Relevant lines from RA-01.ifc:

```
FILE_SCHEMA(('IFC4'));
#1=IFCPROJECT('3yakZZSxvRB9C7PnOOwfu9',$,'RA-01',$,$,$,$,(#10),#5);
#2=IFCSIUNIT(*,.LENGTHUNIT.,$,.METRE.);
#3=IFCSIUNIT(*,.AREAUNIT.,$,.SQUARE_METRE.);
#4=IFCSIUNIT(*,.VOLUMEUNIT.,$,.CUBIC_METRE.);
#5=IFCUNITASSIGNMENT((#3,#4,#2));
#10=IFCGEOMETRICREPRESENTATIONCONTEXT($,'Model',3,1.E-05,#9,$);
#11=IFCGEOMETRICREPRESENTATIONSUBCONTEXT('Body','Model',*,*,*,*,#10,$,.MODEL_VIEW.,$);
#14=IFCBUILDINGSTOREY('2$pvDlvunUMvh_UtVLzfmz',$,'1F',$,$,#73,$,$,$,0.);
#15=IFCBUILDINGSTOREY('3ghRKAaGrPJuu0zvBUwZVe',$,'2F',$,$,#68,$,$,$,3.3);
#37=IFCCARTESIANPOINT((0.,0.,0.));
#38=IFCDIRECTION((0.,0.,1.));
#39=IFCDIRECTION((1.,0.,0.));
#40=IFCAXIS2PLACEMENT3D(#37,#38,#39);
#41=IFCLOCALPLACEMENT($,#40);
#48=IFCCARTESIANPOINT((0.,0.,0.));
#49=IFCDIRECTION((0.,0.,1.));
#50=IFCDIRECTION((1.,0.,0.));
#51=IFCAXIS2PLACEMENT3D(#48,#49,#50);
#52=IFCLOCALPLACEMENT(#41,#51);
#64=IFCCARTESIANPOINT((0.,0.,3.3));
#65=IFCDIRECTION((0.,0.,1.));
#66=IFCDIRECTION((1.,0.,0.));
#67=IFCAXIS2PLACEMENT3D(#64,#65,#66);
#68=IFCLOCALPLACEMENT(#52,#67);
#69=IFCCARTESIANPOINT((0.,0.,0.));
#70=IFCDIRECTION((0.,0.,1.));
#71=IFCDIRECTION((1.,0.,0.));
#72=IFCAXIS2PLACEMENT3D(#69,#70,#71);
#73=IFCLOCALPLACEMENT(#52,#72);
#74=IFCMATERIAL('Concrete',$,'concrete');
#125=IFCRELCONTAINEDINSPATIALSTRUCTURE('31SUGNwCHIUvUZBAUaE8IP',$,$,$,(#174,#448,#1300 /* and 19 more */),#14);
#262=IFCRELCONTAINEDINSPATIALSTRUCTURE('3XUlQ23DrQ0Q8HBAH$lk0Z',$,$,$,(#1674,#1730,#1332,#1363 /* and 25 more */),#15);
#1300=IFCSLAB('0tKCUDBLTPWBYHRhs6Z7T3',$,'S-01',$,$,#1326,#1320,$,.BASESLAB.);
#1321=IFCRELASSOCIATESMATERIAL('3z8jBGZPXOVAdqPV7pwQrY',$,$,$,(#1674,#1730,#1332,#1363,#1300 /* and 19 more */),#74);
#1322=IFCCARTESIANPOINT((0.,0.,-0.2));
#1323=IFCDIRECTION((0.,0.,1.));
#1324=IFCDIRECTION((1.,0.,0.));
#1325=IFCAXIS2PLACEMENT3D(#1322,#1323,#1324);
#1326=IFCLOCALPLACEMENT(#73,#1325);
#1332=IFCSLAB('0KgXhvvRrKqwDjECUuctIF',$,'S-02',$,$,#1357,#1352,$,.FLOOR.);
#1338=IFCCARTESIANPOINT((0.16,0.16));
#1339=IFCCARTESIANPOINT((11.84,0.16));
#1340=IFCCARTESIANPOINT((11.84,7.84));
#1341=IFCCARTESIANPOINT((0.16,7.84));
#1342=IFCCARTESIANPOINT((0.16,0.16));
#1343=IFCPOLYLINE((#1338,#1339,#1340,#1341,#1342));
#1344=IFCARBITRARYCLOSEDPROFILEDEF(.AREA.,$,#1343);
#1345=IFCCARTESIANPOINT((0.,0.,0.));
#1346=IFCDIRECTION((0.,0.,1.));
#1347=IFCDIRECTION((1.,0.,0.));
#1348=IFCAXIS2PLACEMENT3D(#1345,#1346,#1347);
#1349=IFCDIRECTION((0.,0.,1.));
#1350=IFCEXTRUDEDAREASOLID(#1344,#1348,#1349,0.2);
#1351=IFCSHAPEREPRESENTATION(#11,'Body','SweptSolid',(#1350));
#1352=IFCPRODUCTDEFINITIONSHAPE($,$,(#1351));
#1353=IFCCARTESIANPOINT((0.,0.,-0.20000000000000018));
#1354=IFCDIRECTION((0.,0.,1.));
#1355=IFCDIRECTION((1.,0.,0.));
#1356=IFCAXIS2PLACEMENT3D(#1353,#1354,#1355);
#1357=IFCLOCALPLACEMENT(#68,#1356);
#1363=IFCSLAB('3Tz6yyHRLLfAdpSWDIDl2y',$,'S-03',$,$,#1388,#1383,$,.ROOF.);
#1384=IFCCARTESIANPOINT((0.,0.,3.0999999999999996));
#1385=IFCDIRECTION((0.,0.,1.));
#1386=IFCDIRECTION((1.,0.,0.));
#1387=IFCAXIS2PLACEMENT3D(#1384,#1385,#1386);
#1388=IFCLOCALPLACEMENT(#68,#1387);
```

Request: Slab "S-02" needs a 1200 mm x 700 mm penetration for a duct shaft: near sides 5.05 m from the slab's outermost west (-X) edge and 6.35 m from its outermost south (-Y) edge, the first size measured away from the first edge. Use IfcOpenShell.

```python
import numpy as np
import ifcopenshell
import ifcopenshell.api.feature
import ifcopenshell.api.geometry
import ifcopenshell.api.root
import ifcopenshell.geom
import ifcopenshell.util.placement
import ifcopenshell.util.representation
import ifcopenshell.util.shape
import ifcopenshell.util.unit

model = ifcopenshell.open("RA-01.ifc")
unit_scale = ifcopenshell.util.unit.calculate_unit_scale(model)
settings = ifcopenshell.geom.settings()


def volume(element):
    """Net volume in cubic metres, openings subtracted."""
    shape = ifcopenshell.geom.create_shape(settings, element)
    return ifcopenshell.util.shape.get_volume(shape.geometry)


slab = model.by_guid("0KgXhvvRrKqwDjECUuctIF")
before = volume(slab)

# Extent in the slab's own axes, in metres. The edges named are its -X and -Y sides.
slab_shape = ifcopenshell.geom.create_shape(settings, slab)
vertices = ifcopenshell.util.shape.get_vertices(slab_shape.geometry)
x_min, y_min, bottom = vertices.min(axis=0)
top = vertices[:, 2].max()

opening = ifcopenshell.api.root.create_entity(model, ifc_class="IfcOpeningElement", name="Duct shaft opening", predefined_type="OPENING")
context = ifcopenshell.util.representation.get_context(model, "Model", "Body", "MODEL_VIEW")
width, depth = 1.2, 0.7
outline = [(0.0, 0.0), (width, 0.0), (width, depth), (0.0, depth), (0.0, 0.0)]
# Overshoot both faces by 50 mm so the cut is clean.
shape = ifcopenshell.api.geometry.add_slab_representation(
    model, context=context, depth=top - bottom + 0.1, polyline=outline
)
ifcopenshell.api.geometry.assign_representation(model, product=opening, representation=shape)

matrix = ifcopenshell.util.placement.get_local_placement(slab.ObjectPlacement)
matrix[:, 3] = matrix @ np.append(np.array([x_min + 5.05, y_min + 6.35, bottom - 0.05]) / unit_scale, 1.0)
ifcopenshell.api.geometry.edit_object_placement(model, product=opening, matrix=matrix, is_si=False)
ifcopenshell.api.feature.add_feature(model, feature=opening, element=slab)

after = volume(slab)

print(f"slab volume {before:.3f} -> {after:.3f} m3")

model.write("RA-01_edited.ifc")
```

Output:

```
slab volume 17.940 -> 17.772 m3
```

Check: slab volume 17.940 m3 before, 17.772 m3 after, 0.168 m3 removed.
